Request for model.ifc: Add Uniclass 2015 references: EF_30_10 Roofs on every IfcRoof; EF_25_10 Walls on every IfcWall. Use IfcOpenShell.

First a look at what the model holds.

```python
import ifcopenshell

model = ifcopenshell.open("model.ifc")
print(model.schema)
print("classifications:", [c.Name for c in model.by_type("IfcClassification")])
for ifc_class in ("IfcDoor", "IfcRoof", "IfcStair", "IfcWall", "IfcWindow"):
    print(ifc_class, len(model.by_type(ifc_class)))
```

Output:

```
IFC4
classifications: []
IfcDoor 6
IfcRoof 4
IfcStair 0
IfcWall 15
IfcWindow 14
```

```python
import ifcopenshell
import ifcopenshell.api.classification

model = ifcopenshell.open("model.ifc")

system = ifcopenshell.api.classification.add_classification(model, classification="Uniclass 2015")

codes = {
    "IfcRoof": ("EF_30_10", "Roofs"),
    "IfcWall": ("EF_25_10", "Walls"),
}
for ifc_class, (code, name) in codes.items():
    products = model.by_type(ifc_class)
    ifcopenshell.api.classification.add_reference(
        model, products=products, classification=system, identification=code, name=name
    )
    print(code, len(products))

model.write("model_rev.ifc")
```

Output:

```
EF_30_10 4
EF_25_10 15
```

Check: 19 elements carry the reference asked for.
